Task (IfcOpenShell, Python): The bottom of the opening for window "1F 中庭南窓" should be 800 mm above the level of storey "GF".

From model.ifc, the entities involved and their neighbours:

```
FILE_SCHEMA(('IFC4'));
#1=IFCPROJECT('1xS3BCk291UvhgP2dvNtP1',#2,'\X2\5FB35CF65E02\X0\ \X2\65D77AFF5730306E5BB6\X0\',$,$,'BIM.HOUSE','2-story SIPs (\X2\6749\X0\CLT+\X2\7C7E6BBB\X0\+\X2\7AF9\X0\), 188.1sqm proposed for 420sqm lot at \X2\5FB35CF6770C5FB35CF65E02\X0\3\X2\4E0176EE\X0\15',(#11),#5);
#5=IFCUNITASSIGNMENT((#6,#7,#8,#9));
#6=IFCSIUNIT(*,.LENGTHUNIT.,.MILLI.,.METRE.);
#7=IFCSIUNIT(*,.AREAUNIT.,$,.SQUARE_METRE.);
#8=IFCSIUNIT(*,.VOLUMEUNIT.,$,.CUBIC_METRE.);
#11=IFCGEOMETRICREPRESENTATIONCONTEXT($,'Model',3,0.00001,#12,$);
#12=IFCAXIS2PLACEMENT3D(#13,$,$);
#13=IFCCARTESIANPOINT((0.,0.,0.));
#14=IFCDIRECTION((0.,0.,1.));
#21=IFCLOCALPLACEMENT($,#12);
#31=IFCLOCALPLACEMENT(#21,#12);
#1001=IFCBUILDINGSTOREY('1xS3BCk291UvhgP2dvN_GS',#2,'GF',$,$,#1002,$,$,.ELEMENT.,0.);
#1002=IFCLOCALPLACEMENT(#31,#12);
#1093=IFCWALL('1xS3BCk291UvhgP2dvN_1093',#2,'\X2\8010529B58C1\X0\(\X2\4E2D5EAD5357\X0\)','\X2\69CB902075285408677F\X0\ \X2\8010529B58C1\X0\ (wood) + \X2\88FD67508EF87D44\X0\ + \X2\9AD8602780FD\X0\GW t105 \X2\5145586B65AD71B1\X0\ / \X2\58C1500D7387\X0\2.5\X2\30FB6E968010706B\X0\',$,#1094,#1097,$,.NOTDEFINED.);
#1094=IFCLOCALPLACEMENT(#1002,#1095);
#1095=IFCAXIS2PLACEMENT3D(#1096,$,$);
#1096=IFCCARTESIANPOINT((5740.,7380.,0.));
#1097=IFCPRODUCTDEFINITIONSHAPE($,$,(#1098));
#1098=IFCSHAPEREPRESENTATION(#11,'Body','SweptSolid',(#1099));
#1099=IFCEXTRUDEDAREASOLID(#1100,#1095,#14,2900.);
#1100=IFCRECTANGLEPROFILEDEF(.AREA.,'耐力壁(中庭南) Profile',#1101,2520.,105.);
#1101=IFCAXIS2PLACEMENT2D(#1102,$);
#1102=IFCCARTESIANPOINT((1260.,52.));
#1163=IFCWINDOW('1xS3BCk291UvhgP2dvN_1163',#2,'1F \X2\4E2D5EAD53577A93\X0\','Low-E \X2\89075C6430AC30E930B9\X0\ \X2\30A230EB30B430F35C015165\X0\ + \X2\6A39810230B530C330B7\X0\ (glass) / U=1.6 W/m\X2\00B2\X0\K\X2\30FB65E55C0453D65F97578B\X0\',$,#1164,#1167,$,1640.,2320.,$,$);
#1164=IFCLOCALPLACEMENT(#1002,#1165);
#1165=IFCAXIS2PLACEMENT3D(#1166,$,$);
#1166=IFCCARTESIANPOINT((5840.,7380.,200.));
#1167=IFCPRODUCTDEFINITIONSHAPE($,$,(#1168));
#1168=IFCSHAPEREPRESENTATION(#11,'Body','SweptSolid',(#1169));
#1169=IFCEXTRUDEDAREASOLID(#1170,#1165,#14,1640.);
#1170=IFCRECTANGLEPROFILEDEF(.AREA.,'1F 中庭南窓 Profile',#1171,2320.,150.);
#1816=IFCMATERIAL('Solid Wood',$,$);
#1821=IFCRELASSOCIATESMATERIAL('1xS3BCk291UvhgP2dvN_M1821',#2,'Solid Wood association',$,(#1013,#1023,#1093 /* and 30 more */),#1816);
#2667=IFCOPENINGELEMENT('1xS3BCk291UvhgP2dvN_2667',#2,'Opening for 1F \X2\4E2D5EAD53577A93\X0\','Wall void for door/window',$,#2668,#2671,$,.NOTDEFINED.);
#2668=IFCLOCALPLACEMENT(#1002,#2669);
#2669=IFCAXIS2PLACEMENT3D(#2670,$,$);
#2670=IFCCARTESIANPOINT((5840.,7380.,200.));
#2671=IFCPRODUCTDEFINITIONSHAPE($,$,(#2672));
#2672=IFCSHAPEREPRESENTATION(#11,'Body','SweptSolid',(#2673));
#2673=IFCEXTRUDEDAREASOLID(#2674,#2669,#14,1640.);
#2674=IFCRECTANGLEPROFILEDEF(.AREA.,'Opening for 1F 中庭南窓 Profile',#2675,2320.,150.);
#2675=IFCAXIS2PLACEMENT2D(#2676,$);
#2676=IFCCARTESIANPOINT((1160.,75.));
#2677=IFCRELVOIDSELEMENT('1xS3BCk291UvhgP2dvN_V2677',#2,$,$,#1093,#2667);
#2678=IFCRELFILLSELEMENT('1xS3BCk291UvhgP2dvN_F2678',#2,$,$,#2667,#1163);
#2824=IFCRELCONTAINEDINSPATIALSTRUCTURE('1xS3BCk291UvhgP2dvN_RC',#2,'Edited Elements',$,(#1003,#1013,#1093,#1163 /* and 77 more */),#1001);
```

```python
import numpy as np
import ifcopenshell
import ifcopenshell.api.geometry
import ifcopenshell.geom
import ifcopenshell.util.element
import ifcopenshell.util.placement
import ifcopenshell.util.shape
import ifcopenshell.util.unit

model = ifcopenshell.open("model.ifc")
unit_scale = ifcopenshell.util.unit.calculate_unit_scale(model)

window = model.by_guid("1xS3BCk291UvhgP2dvN_1163")
opening = window.FillsVoids[0].RelatingOpeningElement
storey = ifcopenshell.util.element.get_container(window, ifc_class="IfcBuildingStorey")
level = ifcopenshell.util.placement.get_local_placement(storey.ObjectPlacement)[2, 3]

# The opening's origin need not be at the sill, so measure its lowest point.
shape = ifcopenshell.geom.create_shape(ifcopenshell.geom.settings(), opening)
bottom = ifcopenshell.util.shape.get_shape_bottom_elevation(shape, shape.geometry) / unit_scale
dz = level + 0.8 / unit_scale - bottom

shift = np.array([0.0, 0.0, dz])
# The window is not placed relative to its opening, so move both.
for product in (opening, window):
    matrix = ifcopenshell.util.placement.get_local_placement(product.ObjectPlacement)
    matrix[:3, 3] += shift
    ifcopenshell.api.geometry.edit_object_placement(model, product=product, matrix=matrix, is_si=False)

print(f"moved by {dz * unit_scale:+.3f} m")

model.write("model_v2.ifc")
```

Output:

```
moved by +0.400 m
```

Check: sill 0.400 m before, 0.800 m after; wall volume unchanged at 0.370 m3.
